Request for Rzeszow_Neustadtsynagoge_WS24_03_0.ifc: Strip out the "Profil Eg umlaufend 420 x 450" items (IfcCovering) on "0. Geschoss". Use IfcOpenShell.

First a look at what the model holds.

```python
import ifcopenshell
import ifcopenshell.util.element

model = ifcopenshell.open("Rzeszow_Neustadtsynagoge_WS24_03_0.ifc")
print(model.schema)
storey = next(s for s in model.by_type("IfcBuildingStorey") if s.Name == "0. Geschoss")
coverings = [e for e in ifcopenshell.util.element.get_decomposition(storey) if e.is_a("IfcCovering")]
seen = {}
for e in coverings:
    element_type = ifcopenshell.util.element.get_type(e)
    name = element_type.Name if element_type not in (None, e) else None
    seen[name] = seen.get(name, 0) + 1
for name, count in sorted(seen.items(), key=str):
    print(count, "x", name)
```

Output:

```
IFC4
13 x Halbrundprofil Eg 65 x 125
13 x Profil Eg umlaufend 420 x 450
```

```python
import ifcopenshell
import ifcopenshell.api.root
import ifcopenshell.util.element

model = ifcopenshell.open("Rzeszow_Neustadtsynagoge_WS24_03_0.ifc")

storey = next(s for s in model.by_type("IfcBuildingStorey") if s.Name == "0. Geschoss")
coverings = [e for e in ifcopenshell.util.element.get_decomposition(storey) if e.is_a("IfcCovering")]
targets = [e for e in coverings if (t := ifcopenshell.util.element.get_type(e)) not in (None, e) and t.Name == "Profil Eg umlaufend 420 x 450"]

for e in targets:
    ifcopenshell.api.root.remove_product(model, product=e)
print(len(targets), "removed")

model.write("Rzeszow_Neustadtsynagoge_WS24_03_0_edited.ifc")
```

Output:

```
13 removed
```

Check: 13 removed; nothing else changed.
